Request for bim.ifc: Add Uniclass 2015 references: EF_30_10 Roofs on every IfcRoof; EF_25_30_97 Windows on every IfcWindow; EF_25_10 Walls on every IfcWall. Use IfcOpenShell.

First a look at what the model holds.

```python
import ifcopenshell

model = ifcopenshell.open("bim.ifc")
print(model.schema)
print("classifications:", [c.Name for c in model.by_type("IfcClassification")])
for ifc_class in ("IfcDoor", "IfcRoof", "IfcStair", "IfcWall", "IfcWindow"):
    print(ifc_class, len(model.by_type(ifc_class)))
```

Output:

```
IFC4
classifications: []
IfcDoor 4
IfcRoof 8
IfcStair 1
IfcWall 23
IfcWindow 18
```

```python
import ifcopenshell
import ifcopenshell.api.classification

model = ifcopenshell.open("bim.ifc")

system = ifcopenshell.api.classification.add_classification(model, classification="Uniclass 2015")

codes = {
    "IfcRoof": ("EF_30_10", "Roofs"),
    "IfcWindow": ("EF_25_30_97", "Windows"),
    "IfcWall": ("EF_25_10", "Walls"),
}
for ifc_class, (code, name) in codes.items():
    products = model.by_type(ifc_class)
    ifcopenshell.api.classification.add_reference(
        model, products=products, classification=system, identification=code, name=name
    )
    print(code, len(products))

model.write("bim-out.ifc")
```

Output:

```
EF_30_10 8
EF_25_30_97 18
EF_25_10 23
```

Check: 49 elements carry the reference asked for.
